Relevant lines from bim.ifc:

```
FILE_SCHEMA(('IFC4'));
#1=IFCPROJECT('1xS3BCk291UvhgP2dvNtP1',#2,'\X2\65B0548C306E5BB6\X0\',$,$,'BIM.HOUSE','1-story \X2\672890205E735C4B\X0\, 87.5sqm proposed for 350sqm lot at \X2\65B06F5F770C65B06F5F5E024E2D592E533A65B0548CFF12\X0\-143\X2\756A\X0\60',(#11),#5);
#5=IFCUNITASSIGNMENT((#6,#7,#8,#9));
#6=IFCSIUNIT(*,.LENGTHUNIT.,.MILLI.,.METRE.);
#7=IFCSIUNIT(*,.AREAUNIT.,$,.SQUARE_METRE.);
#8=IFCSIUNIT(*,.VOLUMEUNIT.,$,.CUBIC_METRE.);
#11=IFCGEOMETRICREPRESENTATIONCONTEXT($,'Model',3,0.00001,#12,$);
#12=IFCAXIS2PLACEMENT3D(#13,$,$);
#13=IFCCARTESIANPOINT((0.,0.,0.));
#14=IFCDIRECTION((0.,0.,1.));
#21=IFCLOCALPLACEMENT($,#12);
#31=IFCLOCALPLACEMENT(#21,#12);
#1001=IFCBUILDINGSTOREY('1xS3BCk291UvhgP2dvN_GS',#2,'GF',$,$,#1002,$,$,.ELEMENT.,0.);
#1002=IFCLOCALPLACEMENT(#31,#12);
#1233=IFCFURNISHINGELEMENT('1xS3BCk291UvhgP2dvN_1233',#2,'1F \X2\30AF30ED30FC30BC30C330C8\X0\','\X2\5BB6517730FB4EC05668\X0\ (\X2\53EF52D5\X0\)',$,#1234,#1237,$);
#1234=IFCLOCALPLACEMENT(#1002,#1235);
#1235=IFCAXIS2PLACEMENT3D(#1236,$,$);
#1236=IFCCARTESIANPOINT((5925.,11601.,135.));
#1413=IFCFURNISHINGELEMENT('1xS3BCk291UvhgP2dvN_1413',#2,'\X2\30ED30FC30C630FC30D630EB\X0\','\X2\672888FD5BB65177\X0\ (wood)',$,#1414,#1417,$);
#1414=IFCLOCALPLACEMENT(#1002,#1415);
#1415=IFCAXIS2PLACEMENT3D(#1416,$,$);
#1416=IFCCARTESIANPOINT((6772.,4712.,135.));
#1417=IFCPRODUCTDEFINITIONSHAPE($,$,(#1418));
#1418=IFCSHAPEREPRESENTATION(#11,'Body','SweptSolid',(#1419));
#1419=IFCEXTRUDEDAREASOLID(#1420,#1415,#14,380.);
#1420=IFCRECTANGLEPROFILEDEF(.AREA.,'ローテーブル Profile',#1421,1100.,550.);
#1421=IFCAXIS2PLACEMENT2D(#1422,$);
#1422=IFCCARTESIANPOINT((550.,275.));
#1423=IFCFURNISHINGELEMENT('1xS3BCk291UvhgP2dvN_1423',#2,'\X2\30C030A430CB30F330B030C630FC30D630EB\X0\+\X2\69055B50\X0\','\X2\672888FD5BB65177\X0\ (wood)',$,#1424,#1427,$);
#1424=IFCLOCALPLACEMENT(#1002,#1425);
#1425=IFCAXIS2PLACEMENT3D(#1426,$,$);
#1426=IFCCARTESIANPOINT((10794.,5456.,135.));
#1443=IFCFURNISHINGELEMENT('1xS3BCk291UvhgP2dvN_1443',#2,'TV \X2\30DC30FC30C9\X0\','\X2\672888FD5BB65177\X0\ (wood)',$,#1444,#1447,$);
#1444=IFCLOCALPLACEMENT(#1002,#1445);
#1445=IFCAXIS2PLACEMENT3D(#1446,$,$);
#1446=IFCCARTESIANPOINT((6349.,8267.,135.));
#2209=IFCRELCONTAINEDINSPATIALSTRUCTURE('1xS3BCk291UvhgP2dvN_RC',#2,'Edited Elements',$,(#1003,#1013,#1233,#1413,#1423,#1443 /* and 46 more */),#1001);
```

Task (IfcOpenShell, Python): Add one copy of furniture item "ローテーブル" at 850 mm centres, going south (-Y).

```python
import numpy as np
import ifcopenshell
import ifcopenshell.api.geometry
import ifcopenshell.api.root
import ifcopenshell.util.element
import ifcopenshell.util.placement
import ifcopenshell.util.unit

model = ifcopenshell.open("bim.ifc")
unit_scale = ifcopenshell.util.unit.calculate_unit_scale(model)


def reuse_history(source, copy):
    """copy_class also copies each property set's owner history, people and application; keep the originals."""
    for rel in copy.IsDefinedBy:
        if rel.is_a("IfcRelDefinesByProperties") and (history := rel.RelatingPropertyDefinition.OwnerHistory):
            rel.RelatingPropertyDefinition.OwnerHistory = source.OwnerHistory
            ifcopenshell.util.element.remove_deep2(model, history)


source = model.by_guid("1xS3BCk291UvhgP2dvN_1413")
base = ifcopenshell.util.placement.get_local_placement(source.ObjectPlacement)
step = np.array([0.0, -1.0, 0.0]) * 0.85 / unit_scale

for i in range(1, 2):
    copy = ifcopenshell.api.root.copy_class(model, product=source)
    copy.Representation = ifcopenshell.util.element.copy_deep(
        model, source.Representation, exclude=["IfcGeometricRepresentationContext", "IfcRepresentationMap"]
    )
    reuse_history(source, copy)
    matrix = base.copy()
    matrix[:3, 3] += i * step
    print("added at", matrix[:3, 3].round(3) + 0.0)
    ifcopenshell.api.geometry.edit_object_placement(model, product=copy, matrix=matrix, is_si=False)

model.write("bim-out.ifc")
```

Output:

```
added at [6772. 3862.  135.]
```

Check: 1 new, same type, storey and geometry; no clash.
